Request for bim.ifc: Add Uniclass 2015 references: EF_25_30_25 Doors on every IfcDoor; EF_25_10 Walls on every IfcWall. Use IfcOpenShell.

First a look at what the model holds.

```python
import ifcopenshell

model = ifcopenshell.open("bim.ifc")
print(model.schema)
print("classifications:", [c.Name for c in model.by_type("IfcClassification")])
for ifc_class in ("IfcDoor", "IfcRoof", "IfcStair", "IfcWall", "IfcWindow"):
    print(ifc_class, len(model.by_type(ifc_class)))
```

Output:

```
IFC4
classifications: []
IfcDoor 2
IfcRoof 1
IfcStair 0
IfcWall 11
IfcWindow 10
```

```python
import ifcopenshell
import ifcopenshell.api.classification

model = ifcopenshell.open("bim.ifc")

system = ifcopenshell.api.classification.add_classification(model, classification="Uniclass 2015")

codes = {
    "IfcDoor": ("EF_25_30_25", "Doors"),
    "IfcWall": ("EF_25_10", "Walls"),
}
for ifc_class, (code, name) in codes.items():
    products = model.by_type(ifc_class)
    ifcopenshell.api.classification.add_reference(
        model, products=products, classification=system, identification=code, name=name
    )
    print(code, len(products))

model.write("bim_edited.ifc")
```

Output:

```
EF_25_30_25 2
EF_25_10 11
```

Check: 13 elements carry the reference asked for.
